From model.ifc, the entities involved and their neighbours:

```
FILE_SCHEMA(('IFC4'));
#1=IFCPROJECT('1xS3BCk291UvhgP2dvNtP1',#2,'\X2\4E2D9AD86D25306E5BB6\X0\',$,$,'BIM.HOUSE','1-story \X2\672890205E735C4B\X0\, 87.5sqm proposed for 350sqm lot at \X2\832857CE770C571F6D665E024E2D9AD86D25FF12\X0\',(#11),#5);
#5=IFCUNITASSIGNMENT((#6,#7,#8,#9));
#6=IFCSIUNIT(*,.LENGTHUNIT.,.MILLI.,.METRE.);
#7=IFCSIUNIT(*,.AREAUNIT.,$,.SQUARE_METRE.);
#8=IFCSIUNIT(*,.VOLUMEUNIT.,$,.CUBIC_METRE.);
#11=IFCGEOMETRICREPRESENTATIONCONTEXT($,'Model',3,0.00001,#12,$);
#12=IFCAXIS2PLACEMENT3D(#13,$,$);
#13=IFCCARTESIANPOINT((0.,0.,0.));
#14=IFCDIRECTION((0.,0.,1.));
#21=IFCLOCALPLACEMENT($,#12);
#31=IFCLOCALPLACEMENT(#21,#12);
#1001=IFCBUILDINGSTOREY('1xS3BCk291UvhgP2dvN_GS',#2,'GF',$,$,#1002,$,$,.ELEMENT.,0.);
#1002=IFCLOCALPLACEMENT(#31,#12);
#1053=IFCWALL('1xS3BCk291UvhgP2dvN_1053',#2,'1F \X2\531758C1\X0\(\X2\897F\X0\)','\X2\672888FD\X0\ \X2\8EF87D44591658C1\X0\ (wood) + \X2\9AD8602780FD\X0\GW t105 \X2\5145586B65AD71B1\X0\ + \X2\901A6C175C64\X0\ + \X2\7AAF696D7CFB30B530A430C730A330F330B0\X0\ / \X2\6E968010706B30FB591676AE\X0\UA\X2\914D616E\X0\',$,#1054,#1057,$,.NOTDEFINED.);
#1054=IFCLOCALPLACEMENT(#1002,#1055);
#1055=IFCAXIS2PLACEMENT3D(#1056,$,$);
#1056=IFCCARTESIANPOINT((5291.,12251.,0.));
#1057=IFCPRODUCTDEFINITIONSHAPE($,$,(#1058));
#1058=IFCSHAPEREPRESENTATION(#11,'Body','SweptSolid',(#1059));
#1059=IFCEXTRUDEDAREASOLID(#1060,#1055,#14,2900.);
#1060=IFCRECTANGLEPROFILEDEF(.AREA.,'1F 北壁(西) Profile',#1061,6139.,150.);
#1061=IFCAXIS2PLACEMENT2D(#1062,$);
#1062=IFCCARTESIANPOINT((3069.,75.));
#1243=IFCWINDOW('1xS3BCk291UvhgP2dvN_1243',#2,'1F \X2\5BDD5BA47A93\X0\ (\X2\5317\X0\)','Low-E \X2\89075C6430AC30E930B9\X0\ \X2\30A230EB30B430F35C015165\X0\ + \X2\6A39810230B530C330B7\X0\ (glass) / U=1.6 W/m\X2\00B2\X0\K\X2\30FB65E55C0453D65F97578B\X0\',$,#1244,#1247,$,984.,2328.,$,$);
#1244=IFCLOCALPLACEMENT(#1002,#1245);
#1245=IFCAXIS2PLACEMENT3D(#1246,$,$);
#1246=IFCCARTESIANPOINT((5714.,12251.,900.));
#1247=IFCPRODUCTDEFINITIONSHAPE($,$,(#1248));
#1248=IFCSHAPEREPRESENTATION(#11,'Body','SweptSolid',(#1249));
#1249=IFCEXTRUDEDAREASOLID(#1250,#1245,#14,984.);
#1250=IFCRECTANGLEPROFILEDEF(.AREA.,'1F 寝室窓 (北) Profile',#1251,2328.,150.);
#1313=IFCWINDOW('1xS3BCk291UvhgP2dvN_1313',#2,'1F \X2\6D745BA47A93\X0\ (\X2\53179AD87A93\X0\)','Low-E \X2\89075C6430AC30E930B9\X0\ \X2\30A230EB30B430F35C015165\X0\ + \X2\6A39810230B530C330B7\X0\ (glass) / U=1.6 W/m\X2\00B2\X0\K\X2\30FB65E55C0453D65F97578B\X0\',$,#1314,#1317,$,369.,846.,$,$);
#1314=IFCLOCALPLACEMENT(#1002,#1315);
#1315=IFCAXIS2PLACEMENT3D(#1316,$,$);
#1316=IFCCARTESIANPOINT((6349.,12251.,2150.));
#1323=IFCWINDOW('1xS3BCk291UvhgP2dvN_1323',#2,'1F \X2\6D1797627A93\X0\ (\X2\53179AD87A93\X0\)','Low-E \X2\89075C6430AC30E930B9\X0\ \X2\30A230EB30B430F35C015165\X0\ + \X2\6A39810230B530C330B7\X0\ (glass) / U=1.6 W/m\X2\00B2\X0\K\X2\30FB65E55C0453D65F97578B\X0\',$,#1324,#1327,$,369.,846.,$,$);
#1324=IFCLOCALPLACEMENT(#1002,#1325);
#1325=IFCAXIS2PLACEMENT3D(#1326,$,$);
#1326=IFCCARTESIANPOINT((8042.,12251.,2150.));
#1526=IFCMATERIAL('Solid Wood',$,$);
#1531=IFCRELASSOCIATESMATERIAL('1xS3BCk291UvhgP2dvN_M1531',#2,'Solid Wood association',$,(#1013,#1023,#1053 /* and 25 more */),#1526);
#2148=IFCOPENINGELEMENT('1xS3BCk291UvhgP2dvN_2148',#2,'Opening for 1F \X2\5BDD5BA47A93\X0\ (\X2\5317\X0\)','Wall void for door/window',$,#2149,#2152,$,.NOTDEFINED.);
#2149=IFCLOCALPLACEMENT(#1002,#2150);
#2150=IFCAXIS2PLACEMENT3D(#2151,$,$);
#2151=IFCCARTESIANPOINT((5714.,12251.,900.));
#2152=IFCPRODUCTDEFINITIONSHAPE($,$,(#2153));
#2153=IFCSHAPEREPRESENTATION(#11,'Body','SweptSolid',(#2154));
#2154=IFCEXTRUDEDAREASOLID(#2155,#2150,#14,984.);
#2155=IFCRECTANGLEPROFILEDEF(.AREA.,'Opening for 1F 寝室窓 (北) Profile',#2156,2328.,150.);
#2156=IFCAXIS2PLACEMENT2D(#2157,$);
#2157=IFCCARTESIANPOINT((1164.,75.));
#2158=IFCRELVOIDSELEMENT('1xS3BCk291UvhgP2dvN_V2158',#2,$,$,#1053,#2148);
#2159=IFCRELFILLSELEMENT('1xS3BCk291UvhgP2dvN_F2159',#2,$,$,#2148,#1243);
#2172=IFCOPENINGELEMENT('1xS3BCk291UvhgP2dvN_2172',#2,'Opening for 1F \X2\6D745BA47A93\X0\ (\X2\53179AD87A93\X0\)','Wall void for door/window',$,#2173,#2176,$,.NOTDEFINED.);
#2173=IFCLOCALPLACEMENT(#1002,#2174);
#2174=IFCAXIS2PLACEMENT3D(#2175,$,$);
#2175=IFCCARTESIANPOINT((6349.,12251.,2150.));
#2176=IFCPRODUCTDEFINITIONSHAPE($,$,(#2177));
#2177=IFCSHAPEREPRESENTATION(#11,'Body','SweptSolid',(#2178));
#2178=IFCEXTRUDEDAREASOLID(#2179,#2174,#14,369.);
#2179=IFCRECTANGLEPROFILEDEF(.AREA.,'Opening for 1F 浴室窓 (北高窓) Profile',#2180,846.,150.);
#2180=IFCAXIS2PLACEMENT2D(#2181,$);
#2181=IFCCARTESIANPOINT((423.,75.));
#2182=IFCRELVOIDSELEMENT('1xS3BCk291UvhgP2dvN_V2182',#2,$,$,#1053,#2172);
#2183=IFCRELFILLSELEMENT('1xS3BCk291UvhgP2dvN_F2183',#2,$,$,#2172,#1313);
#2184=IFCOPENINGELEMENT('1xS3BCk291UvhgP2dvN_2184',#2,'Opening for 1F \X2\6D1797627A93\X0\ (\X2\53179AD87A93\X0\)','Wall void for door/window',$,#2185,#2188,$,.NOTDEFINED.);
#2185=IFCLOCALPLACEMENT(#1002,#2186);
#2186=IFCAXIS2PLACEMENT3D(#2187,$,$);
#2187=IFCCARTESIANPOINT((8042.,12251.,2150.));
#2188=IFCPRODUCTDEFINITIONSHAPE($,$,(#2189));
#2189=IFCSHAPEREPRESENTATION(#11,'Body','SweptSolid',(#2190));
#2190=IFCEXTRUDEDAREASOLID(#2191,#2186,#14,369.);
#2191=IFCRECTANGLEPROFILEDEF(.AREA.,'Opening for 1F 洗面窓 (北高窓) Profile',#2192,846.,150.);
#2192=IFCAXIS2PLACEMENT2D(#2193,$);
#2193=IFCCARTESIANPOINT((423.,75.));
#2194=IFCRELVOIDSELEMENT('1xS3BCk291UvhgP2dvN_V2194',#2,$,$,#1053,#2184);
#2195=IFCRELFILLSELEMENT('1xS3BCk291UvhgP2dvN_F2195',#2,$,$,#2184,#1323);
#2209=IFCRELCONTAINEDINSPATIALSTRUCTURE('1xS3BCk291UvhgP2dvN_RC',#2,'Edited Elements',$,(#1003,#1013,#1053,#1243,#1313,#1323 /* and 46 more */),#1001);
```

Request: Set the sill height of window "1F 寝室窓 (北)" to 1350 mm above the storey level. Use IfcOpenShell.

```python
import numpy as np
import ifcopenshell
import ifcopenshell.api.geometry
import ifcopenshell.geom
import ifcopenshell.util.element
import ifcopenshell.util.placement
import ifcopenshell.util.shape
import ifcopenshell.util.unit

model = ifcopenshell.open("model.ifc")
unit_scale = ifcopenshell.util.unit.calculate_unit_scale(model)

window = model.by_guid("1xS3BCk291UvhgP2dvN_1243")
opening = window.FillsVoids[0].RelatingOpeningElement
storey = ifcopenshell.util.element.get_container(window, ifc_class="IfcBuildingStorey")
level = ifcopenshell.util.placement.get_local_placement(storey.ObjectPlacement)[2, 3]

# The opening's origin need not be at the sill, so measure its lowest point.
shape = ifcopenshell.geom.create_shape(ifcopenshell.geom.settings(), opening)
bottom = ifcopenshell.util.shape.get_shape_bottom_elevation(shape, shape.geometry) / unit_scale
dz = level + 1.35 / unit_scale - bottom

shift = np.array([0.0, 0.0, dz])
# The window is not placed relative to its opening, so move both.
for product in (opening, window):
    matrix = ifcopenshell.util.placement.get_local_placement(product.ObjectPlacement)
    matrix[:3, 3] += shift
    ifcopenshell.api.geometry.edit_object_placement(model, product=product, matrix=matrix, is_si=False)

print(f"moved by {dz * unit_scale:+.3f} m")

model.write("model_updated.ifc")
```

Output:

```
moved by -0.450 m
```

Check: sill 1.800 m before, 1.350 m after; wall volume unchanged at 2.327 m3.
